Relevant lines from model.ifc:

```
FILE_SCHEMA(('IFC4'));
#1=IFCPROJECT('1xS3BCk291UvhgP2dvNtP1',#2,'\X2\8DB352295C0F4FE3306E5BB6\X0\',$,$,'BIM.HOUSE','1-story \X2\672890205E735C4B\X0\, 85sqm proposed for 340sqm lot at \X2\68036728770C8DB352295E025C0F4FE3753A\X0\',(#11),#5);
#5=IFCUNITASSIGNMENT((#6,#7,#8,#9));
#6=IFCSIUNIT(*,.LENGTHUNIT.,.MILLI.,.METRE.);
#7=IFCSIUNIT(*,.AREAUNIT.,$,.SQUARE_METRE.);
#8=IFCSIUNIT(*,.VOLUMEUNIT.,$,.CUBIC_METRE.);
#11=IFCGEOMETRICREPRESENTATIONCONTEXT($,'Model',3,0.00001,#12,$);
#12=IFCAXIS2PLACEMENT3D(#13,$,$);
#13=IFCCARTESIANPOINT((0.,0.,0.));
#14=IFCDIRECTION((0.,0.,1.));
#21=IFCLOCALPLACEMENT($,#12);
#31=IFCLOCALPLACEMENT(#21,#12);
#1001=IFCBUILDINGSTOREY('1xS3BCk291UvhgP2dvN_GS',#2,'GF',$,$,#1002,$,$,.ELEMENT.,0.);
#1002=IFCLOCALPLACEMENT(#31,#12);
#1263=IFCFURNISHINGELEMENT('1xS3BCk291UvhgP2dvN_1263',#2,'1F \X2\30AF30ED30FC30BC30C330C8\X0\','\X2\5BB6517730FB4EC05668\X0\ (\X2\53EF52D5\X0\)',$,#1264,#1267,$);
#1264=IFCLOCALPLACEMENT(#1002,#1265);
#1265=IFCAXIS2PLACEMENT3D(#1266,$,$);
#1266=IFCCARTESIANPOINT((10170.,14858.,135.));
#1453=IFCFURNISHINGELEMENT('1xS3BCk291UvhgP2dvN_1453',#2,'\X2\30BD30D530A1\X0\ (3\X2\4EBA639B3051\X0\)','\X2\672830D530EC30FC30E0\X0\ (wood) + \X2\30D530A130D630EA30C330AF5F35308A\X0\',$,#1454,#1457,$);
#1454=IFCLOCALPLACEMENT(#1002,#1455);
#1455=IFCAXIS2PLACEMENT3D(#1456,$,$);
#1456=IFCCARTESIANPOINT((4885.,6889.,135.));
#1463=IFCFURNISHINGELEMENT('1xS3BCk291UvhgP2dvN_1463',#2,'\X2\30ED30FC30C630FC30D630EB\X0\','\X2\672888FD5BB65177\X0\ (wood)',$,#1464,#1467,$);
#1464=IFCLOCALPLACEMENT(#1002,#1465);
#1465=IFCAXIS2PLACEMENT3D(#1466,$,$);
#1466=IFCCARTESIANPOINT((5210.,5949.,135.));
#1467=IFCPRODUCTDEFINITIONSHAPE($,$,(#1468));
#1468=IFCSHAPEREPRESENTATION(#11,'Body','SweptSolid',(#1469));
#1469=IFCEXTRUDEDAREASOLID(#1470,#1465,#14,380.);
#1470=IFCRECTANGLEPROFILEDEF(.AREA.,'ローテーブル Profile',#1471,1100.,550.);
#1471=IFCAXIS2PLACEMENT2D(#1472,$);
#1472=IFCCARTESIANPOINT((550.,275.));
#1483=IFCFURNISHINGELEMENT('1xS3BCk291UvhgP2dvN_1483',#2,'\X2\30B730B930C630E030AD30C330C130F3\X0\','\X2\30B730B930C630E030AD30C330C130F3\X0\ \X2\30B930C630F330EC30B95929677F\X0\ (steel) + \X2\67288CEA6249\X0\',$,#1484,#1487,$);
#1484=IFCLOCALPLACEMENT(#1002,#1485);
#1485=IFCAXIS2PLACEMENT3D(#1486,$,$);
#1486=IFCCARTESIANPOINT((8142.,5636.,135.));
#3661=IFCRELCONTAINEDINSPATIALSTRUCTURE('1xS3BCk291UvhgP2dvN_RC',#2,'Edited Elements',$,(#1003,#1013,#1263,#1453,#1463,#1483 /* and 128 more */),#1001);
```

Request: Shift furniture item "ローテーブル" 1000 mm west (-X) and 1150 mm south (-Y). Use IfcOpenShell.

```python
import ifcopenshell
import ifcopenshell.api.geometry
import ifcopenshell.util.placement
import ifcopenshell.util.unit

model = ifcopenshell.open("model.ifc")
unit_scale = ifcopenshell.util.unit.calculate_unit_scale(model)

item = model.by_guid("1xS3BCk291UvhgP2dvN_1463")
matrix = ifcopenshell.util.placement.get_local_placement(item.ObjectPlacement)
matrix[0, 3] -= 1 / unit_scale
matrix[1, 3] -= 1.15 / unit_scale
ifcopenshell.api.geometry.edit_object_placement(model, product=item, matrix=matrix, is_si=False)

print(ifcopenshell.util.placement.get_local_placement(item.ObjectPlacement).round(3) + 0.0)

model.write("model-out.ifc")
```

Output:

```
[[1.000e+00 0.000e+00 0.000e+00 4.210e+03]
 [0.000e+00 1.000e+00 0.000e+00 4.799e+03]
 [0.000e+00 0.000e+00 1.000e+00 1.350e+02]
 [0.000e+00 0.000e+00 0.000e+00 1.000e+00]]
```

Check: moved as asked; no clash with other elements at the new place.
